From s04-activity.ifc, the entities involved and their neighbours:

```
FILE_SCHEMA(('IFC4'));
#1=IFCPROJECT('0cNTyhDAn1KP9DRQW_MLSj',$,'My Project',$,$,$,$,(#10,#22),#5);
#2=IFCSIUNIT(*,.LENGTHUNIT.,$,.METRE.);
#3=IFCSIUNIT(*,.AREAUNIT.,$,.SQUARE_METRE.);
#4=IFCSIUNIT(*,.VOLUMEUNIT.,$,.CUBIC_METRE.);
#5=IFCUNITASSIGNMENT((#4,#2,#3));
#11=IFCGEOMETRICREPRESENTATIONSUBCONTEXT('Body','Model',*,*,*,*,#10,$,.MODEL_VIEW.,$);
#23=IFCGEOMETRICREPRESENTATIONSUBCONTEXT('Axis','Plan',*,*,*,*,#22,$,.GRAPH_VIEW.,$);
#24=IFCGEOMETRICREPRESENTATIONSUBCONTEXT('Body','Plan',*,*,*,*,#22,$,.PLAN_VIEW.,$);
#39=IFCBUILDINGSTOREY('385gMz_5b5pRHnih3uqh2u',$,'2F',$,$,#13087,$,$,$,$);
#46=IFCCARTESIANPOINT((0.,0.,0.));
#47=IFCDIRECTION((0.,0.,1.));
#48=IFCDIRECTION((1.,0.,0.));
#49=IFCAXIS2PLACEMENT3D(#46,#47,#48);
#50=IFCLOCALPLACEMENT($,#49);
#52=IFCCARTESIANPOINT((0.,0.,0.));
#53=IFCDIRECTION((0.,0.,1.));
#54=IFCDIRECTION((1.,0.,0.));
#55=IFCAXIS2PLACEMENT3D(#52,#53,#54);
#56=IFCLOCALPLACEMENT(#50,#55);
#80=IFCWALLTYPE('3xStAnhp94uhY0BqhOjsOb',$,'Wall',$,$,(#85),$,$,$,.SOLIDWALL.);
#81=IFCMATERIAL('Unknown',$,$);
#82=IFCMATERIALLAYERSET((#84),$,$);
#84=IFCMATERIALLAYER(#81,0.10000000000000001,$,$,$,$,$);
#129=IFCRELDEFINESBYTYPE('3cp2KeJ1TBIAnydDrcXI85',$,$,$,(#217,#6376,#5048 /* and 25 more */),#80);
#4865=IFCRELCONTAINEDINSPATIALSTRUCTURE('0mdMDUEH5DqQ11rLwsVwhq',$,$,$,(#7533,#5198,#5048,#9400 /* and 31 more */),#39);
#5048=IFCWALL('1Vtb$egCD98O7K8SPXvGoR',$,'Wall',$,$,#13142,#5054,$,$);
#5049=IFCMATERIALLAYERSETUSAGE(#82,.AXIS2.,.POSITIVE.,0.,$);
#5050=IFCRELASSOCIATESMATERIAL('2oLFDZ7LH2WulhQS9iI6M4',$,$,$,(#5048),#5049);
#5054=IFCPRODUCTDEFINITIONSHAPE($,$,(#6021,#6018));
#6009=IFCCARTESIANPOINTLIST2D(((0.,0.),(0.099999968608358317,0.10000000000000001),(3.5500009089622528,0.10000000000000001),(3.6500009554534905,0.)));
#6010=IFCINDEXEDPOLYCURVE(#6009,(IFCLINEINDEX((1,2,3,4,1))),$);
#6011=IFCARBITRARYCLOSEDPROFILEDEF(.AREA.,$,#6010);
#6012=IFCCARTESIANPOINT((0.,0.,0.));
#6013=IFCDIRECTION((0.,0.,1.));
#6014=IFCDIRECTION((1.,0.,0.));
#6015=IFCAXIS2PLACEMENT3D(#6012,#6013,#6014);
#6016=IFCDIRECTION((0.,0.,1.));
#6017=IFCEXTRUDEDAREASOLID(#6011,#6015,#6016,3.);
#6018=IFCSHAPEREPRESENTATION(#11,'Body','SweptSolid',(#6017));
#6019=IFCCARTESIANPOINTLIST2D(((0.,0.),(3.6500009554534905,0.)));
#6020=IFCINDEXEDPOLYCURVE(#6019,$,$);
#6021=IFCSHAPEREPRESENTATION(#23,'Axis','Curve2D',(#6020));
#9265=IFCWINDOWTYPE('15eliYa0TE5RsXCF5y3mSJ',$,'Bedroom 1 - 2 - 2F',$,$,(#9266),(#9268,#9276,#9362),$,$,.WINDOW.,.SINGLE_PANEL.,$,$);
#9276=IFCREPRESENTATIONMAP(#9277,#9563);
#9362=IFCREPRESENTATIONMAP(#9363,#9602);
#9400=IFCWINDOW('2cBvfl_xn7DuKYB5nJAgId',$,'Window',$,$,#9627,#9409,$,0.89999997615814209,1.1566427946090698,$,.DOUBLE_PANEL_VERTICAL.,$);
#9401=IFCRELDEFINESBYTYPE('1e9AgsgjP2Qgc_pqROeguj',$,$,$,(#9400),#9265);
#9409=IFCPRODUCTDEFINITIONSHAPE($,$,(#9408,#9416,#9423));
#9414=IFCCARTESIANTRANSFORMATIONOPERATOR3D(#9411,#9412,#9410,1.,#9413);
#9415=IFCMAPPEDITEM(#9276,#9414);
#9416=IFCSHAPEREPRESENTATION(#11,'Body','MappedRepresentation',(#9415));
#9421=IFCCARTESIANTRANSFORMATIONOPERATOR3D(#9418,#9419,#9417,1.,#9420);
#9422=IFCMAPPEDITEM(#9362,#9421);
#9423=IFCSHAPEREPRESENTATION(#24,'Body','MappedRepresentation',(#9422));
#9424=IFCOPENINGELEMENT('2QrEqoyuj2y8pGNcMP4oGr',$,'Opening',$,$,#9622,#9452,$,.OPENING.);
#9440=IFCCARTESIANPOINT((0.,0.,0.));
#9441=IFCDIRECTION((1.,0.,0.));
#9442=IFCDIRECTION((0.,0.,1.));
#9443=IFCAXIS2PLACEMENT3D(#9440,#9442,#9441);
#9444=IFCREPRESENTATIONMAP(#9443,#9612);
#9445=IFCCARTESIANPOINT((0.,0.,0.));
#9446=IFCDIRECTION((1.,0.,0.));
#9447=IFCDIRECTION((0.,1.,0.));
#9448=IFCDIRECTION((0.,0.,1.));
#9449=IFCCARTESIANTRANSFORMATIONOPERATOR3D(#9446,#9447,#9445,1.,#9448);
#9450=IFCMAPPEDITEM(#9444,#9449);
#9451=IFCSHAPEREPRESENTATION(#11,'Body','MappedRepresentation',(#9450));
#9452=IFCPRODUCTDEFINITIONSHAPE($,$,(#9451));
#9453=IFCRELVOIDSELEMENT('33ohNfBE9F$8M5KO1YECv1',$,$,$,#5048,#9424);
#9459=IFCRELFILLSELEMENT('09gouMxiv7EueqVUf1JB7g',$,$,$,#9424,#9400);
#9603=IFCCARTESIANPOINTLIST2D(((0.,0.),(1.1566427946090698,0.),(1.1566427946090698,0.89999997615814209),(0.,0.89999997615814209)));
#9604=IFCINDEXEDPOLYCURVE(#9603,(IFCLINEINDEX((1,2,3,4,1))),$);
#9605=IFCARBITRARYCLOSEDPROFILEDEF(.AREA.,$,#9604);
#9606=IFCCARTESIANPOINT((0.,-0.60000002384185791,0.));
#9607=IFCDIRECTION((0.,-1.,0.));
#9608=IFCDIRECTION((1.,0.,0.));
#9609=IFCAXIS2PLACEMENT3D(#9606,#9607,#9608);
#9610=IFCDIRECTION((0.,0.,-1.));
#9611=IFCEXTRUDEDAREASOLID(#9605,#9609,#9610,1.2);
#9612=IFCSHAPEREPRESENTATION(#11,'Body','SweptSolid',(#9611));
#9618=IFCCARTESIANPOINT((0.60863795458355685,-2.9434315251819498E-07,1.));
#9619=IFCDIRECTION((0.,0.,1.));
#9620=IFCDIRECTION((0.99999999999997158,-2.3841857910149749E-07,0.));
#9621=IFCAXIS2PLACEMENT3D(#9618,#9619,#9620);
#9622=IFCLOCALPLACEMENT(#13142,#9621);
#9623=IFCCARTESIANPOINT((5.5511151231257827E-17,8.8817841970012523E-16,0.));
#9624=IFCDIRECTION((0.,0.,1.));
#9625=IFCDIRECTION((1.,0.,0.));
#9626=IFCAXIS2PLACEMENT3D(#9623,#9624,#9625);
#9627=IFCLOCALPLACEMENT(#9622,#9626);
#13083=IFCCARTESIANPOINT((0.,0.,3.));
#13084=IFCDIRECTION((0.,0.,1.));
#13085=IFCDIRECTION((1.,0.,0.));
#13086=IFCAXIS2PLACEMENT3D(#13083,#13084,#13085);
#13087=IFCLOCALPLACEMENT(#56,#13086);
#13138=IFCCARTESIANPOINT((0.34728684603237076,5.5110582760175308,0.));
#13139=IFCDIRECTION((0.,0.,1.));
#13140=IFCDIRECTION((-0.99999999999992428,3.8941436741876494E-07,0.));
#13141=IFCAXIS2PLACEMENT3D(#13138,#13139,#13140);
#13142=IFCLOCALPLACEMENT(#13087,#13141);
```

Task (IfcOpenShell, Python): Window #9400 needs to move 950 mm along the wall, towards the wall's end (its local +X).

```python
import ifcopenshell
import ifcopenshell.api.geometry
import ifcopenshell.util.placement
import ifcopenshell.util.unit

model = ifcopenshell.open("s04-activity.ifc")
unit_scale = ifcopenshell.util.unit.calculate_unit_scale(model)

window = model.by_guid("2cBvfl_xn7DuKYB5nJAgId")
opening = window.FillsVoids[0].RelatingOpeningElement
wall = opening.VoidsElements[0].RelatingBuildingElement

wall_matrix = ifcopenshell.util.placement.get_local_placement(wall.ObjectPlacement)
shift = wall_matrix[:3, 0] * 0.95 / unit_scale
before = ifcopenshell.util.placement.get_local_placement(window.ObjectPlacement)[:3, 3].copy()

# The window is placed relative to its opening, so it follows when the opening moves.
matrix = ifcopenshell.util.placement.get_local_placement(opening.ObjectPlacement)
matrix[:3, 3] += shift
ifcopenshell.api.geometry.edit_object_placement(
    model, product=opening, matrix=matrix, is_si=False, should_transform_children=True
)

after = ifcopenshell.util.placement.get_local_placement(window.ObjectPlacement)[:3, 3]
print("window moved by", (after - before).round(3) + 0.0)

model.write("s04-activity_edited.ifc")
```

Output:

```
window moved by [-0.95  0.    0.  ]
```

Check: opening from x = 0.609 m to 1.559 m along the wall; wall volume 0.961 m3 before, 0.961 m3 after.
